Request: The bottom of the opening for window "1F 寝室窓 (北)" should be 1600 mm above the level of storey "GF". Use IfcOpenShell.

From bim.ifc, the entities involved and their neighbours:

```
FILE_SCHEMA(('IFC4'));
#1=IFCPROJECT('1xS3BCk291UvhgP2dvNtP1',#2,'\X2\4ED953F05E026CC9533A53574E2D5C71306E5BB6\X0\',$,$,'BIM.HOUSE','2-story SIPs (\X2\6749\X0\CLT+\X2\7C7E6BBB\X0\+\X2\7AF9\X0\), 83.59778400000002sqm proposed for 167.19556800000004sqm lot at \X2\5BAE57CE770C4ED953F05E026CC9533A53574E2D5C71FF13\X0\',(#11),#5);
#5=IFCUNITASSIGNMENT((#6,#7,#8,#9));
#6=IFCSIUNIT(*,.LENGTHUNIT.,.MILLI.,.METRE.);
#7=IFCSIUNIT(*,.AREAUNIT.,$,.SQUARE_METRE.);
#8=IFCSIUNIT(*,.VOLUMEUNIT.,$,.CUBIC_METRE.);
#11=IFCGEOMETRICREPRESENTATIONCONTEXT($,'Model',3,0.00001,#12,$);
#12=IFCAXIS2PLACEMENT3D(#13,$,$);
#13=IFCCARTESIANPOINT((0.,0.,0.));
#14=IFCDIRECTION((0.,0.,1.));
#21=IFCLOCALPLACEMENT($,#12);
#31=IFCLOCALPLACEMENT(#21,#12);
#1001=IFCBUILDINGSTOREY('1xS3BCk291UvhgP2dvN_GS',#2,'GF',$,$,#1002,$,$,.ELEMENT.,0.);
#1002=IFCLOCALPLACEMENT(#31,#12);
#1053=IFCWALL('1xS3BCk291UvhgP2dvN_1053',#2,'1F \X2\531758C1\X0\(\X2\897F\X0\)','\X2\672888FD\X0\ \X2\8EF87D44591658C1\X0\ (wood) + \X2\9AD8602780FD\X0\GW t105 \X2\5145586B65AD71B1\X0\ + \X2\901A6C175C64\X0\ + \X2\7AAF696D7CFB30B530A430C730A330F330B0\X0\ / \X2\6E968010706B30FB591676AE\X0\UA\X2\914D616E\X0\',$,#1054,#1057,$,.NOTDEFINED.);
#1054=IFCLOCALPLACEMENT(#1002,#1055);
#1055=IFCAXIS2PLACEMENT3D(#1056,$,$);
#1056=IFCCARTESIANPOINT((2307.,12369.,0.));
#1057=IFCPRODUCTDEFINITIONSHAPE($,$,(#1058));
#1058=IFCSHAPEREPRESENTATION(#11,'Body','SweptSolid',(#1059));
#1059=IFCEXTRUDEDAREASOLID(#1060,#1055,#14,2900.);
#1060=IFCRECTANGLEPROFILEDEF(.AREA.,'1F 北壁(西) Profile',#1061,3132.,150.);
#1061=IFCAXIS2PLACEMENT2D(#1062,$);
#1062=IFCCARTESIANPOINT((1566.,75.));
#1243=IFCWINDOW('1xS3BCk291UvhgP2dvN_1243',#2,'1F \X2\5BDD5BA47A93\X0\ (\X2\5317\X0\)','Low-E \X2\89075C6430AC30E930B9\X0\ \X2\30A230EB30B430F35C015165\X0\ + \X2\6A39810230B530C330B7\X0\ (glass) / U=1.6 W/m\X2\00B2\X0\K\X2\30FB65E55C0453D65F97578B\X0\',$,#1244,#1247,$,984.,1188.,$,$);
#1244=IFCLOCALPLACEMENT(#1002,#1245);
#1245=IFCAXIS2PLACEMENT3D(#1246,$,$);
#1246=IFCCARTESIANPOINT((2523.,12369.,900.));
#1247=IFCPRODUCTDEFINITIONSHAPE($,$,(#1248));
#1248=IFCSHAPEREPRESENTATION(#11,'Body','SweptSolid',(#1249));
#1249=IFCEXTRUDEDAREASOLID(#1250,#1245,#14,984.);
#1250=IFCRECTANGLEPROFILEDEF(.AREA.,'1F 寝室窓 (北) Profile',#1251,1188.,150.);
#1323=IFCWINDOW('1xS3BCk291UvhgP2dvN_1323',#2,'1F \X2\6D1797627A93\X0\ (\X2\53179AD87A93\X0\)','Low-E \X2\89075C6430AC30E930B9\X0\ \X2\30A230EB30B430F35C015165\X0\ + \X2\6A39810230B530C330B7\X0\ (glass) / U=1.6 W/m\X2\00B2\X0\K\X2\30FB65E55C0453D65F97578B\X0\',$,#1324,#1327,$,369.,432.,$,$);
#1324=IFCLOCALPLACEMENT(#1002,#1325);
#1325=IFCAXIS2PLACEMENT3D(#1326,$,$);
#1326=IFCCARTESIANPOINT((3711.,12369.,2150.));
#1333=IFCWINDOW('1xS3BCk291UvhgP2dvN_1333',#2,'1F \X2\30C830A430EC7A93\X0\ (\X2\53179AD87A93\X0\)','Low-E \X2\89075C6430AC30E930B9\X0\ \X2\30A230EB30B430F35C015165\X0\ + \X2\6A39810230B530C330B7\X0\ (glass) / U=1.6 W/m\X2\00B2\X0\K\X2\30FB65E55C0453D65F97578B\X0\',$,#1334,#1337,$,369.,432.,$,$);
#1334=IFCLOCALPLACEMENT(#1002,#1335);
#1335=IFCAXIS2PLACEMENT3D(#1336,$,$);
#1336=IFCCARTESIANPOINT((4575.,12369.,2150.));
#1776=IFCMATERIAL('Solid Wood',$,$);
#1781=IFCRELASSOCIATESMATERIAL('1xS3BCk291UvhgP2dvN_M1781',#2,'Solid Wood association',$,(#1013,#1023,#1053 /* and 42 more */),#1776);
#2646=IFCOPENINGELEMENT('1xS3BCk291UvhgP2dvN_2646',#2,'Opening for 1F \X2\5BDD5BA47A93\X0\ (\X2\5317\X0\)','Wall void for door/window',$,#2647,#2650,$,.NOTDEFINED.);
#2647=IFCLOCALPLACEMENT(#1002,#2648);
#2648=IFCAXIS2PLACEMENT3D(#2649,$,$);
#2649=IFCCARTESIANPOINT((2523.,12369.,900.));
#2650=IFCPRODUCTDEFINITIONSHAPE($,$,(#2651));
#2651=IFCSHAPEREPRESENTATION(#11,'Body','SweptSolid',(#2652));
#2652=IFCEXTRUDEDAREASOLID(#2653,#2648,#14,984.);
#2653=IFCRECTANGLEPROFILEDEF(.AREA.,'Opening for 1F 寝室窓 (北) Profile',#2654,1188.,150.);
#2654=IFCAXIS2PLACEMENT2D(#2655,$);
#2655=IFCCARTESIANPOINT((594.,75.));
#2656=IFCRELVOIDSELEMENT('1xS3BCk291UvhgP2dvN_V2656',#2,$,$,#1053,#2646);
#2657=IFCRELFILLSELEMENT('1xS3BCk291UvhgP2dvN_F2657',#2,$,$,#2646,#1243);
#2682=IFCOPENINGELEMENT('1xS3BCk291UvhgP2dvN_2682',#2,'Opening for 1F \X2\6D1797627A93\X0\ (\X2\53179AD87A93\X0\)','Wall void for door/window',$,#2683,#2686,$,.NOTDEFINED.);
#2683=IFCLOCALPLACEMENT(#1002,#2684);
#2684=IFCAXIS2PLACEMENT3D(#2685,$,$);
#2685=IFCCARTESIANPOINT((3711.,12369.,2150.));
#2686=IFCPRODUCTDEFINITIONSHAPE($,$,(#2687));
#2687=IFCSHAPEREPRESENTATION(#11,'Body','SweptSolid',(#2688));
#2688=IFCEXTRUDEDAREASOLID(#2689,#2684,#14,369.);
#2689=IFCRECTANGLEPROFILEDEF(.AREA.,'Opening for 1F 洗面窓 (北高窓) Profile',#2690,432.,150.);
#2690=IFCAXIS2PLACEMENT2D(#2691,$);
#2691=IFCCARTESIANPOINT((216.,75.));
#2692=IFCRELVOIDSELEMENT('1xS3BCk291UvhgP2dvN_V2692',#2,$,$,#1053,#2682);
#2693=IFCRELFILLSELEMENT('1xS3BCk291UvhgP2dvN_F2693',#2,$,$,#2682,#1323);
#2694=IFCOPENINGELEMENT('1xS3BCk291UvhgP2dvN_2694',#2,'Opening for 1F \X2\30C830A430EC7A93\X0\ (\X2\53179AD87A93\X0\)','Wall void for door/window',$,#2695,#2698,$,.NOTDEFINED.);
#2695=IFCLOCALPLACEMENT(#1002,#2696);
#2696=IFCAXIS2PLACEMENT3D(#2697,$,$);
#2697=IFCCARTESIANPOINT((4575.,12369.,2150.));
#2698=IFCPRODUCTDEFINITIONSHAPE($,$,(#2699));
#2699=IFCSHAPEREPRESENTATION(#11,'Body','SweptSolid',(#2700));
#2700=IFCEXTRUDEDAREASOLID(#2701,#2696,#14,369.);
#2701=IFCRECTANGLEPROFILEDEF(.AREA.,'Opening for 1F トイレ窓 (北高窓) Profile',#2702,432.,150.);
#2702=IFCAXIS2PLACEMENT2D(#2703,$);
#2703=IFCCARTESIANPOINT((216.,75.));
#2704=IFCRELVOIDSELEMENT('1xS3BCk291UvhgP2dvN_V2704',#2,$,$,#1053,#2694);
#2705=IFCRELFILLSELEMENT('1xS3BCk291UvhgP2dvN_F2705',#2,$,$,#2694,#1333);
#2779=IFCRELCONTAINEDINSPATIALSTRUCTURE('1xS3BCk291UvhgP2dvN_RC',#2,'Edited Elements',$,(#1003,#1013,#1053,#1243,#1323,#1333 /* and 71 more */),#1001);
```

```python
import numpy as np
import ifcopenshell
import ifcopenshell.api.geometry
import ifcopenshell.geom
import ifcopenshell.util.element
import ifcopenshell.util.placement
import ifcopenshell.util.shape
import ifcopenshell.util.unit

model = ifcopenshell.open("bim.ifc")
unit_scale = ifcopenshell.util.unit.calculate_unit_scale(model)

window = model.by_guid("1xS3BCk291UvhgP2dvN_1243")
opening = window.FillsVoids[0].RelatingOpeningElement
storey = ifcopenshell.util.element.get_container(window, ifc_class="IfcBuildingStorey")
level = ifcopenshell.util.placement.get_local_placement(storey.ObjectPlacement)[2, 3]

# The opening's origin need not be at the sill, so measure its lowest point.
shape = ifcopenshell.geom.create_shape(ifcopenshell.geom.settings(), opening)
bottom = ifcopenshell.util.shape.get_shape_bottom_elevation(shape, shape.geometry) / unit_scale
dz = level + 1.6 / unit_scale - bottom

shift = np.array([0.0, 0.0, dz])
# The window is not placed relative to its opening, so move both.
for product in (opening, window):
    matrix = ifcopenshell.util.placement.get_local_placement(product.ObjectPlacement)
    matrix[:3, 3] += shift
    ifcopenshell.api.geometry.edit_object_placement(model, product=product, matrix=matrix, is_si=False)

print(f"moved by {dz * unit_scale:+.3f} m")

model.write("bim_rev.ifc")
```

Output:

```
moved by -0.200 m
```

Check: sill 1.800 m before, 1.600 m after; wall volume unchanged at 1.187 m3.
